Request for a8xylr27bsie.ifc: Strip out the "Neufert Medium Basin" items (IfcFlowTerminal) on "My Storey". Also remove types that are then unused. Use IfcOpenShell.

First a look at what the model holds.

```python
import ifcopenshell
import ifcopenshell.util.element

model = ifcopenshell.open("a8xylr27bsie.ifc")
print(model.schema)
storey = next(s for s in model.by_type("IfcBuildingStorey") if s.Name == "My Storey")
terminals = [e for e in ifcopenshell.util.element.get_decomposition(storey) if e.is_a("IfcFlowTerminal")]
seen = {}
for e in terminals:
    element_type = ifcopenshell.util.element.get_type(e)
    name = element_type.Name if element_type not in (None, e) else None
    seen[name] = seen.get(name, 0) + 1
for name, count in sorted(seen.items(), key=str):
    print(count, "x", name)
```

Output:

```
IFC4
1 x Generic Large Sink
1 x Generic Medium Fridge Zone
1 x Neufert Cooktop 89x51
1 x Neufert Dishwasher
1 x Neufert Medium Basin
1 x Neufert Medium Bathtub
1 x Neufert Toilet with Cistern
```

```python
import ifcopenshell
import ifcopenshell.api.root
import ifcopenshell.util.element

model = ifcopenshell.open("a8xylr27bsie.ifc")

storey = next(s for s in model.by_type("IfcBuildingStorey") if s.Name == "My Storey")
terminals = [e for e in ifcopenshell.util.element.get_decomposition(storey) if e.is_a("IfcFlowTerminal")]
targets = [e for e in terminals if (t := ifcopenshell.util.element.get_type(e)) not in (None, e) and t.Name == "Neufert Medium Basin"]
types = {ifcopenshell.util.element.get_type(e) for e in targets} - {None, *targets}

for e in targets:
    ifcopenshell.api.root.remove_product(model, product=e)
print(len(targets), "removed")

unused = [t for t in types if not ifcopenshell.util.element.get_types(t)]
for t in unused:
    ifcopenshell.api.root.remove_product(model, product=t)
print(len(unused), "unused types removed")

model.write("a8xylr27bsie_edited.ifc")
```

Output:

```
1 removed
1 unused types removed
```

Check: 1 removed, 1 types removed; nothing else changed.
